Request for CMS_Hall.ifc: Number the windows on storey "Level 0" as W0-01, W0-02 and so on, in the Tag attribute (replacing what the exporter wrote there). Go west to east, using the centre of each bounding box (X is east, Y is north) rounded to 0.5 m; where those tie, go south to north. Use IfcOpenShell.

First a look at what the model holds.

```python
import ifcopenshell
import ifcopenshell.util.element
import ifcopenshell.util.placement

model = ifcopenshell.open("CMS_Hall.ifc")
print(model.schema)
storey = next(s for s in model.by_type("IfcBuildingStorey") if s.Name == "Level 0")
windows = [e for e in ifcopenshell.util.element.get_decomposition(storey) if e.is_a("IfcWindow")]
for e in sorted(windows, key=lambda e: e.id()):
    origin = ifcopenshell.util.placement.get_local_placement(e.ObjectPlacement)[:3, 3]
    print(e.id(), e.Tag, e.Name, origin.round(2) + 0.0, sep=" | ")
```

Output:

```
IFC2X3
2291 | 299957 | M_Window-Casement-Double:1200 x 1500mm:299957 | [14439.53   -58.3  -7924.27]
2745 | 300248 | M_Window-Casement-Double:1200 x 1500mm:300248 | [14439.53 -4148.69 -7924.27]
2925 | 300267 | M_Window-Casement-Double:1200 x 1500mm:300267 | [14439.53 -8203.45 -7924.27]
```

```python
import ifcopenshell
import ifcopenshell.geom
import ifcopenshell.util.element
import ifcopenshell.util.shape

model = ifcopenshell.open("CMS_Hall.ifc")
settings = ifcopenshell.geom.settings()
settings.set("use-world-coords", True)


def centre(element):
    shape = ifcopenshell.geom.create_shape(settings, element)
    return ifcopenshell.util.shape.get_bbox_centroid(shape.geometry)


storey = next(s for s in model.by_type("IfcBuildingStorey") if s.Name == "Level 0")
windows = [e for e in ifcopenshell.util.element.get_decomposition(storey) if e.is_a("IfcWindow")]

# Insertion points can sit at a corner or the storey origin, so sort by the geometry (in metres).
centres = {e: centre(e) for e in windows}
windows.sort(key=lambda e: (round(centres[e][0] / 0.5), centres[e][1]))

for i, e in enumerate(windows, start=1):
    number = f"W0-{i:02d}"
    e.Tag = number
    print(e.id(), number)

model.write("CMS_Hall-out.ifc")
```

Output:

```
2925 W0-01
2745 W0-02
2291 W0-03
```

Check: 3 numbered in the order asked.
